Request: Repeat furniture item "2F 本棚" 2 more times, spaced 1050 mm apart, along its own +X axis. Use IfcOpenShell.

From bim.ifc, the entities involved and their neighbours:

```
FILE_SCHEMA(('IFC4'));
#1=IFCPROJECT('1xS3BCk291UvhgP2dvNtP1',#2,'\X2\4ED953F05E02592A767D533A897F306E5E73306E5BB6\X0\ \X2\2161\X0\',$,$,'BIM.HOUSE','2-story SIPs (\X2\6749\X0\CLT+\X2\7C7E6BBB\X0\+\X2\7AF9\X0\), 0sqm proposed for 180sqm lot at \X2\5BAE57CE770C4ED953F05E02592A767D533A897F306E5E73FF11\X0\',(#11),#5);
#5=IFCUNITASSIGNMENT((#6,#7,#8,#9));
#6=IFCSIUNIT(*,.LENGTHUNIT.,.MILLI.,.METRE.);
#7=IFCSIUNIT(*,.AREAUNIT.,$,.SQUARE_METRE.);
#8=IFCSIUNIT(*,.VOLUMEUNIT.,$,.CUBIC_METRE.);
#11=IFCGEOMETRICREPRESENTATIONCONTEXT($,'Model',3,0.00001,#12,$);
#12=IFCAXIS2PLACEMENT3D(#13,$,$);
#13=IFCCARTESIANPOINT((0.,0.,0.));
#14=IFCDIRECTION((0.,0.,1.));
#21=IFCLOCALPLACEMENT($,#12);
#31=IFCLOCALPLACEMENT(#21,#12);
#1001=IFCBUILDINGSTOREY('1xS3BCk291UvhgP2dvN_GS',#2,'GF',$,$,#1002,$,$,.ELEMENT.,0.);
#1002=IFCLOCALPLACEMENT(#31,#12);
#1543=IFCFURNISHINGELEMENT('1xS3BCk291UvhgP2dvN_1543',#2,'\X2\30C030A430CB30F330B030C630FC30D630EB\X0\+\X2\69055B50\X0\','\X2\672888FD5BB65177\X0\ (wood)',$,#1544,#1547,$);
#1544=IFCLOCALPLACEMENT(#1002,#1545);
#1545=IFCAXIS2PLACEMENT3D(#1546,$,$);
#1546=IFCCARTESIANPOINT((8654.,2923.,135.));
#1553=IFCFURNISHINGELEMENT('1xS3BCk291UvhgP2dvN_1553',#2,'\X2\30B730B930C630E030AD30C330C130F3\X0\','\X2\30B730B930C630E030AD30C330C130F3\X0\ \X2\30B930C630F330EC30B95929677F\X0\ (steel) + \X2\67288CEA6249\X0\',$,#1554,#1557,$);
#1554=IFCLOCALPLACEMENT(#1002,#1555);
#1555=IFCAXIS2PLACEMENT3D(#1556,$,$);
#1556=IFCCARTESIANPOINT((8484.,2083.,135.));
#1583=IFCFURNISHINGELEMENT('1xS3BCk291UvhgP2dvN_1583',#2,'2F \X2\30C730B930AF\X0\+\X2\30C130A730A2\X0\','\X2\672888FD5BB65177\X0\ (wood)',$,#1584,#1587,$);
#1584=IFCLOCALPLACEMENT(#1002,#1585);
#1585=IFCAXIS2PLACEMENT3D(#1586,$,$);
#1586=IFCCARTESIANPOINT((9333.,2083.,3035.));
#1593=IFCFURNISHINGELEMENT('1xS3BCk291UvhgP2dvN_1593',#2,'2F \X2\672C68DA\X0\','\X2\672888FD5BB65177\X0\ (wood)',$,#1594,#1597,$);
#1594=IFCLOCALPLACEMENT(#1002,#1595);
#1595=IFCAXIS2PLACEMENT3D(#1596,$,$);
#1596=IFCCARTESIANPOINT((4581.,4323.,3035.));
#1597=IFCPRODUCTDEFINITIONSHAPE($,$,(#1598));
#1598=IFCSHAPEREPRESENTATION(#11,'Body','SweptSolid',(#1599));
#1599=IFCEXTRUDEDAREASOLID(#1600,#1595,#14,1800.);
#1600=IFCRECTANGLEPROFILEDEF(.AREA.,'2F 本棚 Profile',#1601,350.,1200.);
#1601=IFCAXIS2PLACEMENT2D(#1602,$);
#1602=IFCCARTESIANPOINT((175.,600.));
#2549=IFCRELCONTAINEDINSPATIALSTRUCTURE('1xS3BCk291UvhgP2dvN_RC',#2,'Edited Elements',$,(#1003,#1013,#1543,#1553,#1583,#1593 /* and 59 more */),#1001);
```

```python
import ifcopenshell
import ifcopenshell.api.geometry
import ifcopenshell.api.root
import ifcopenshell.util.element
import ifcopenshell.util.placement
import ifcopenshell.util.unit

model = ifcopenshell.open("bim.ifc")
unit_scale = ifcopenshell.util.unit.calculate_unit_scale(model)


def reuse_history(source, copy):
    """copy_class also copies each property set's owner history, people and application; keep the originals."""
    for rel in copy.IsDefinedBy:
        if rel.is_a("IfcRelDefinesByProperties") and (history := rel.RelatingPropertyDefinition.OwnerHistory):
            rel.RelatingPropertyDefinition.OwnerHistory = source.OwnerHistory
            ifcopenshell.util.element.remove_deep2(model, history)


source = model.by_guid("1xS3BCk291UvhgP2dvN_1593")
base = ifcopenshell.util.placement.get_local_placement(source.ObjectPlacement)
step = base[:3, 0] * 1.05 / unit_scale

for i in range(1, 3):
    copy = ifcopenshell.api.root.copy_class(model, product=source)
    copy.Representation = ifcopenshell.util.element.copy_deep(
        model, source.Representation, exclude=["IfcGeometricRepresentationContext", "IfcRepresentationMap"]
    )
    reuse_history(source, copy)
    matrix = base.copy()
    matrix[:3, 3] += i * step
    print("added at", matrix[:3, 3].round(3) + 0.0)
    ifcopenshell.api.geometry.edit_object_placement(model, product=copy, matrix=matrix, is_si=False)

model.write("bim-out.ifc")
```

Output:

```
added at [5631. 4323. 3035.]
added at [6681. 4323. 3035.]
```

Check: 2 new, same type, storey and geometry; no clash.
